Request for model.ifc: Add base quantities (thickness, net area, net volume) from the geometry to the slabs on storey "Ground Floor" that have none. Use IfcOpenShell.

First a look at what the model holds.

```python
import ifcopenshell
import ifcopenshell.util.element
import ifcopenshell.util.unit

model = ifcopenshell.open("model.ifc")
print(model.schema)
for unit_type in ("LENGTHUNIT", "AREAUNIT", "VOLUMEUNIT"):
    print(unit_type, ifcopenshell.util.unit.calculate_unit_scale(model, unit_type))
storey = next(s for s in model.by_type("IfcBuildingStorey") if s.Name == "Ground Floor")
slabs = [e for e in ifcopenshell.util.element.get_decomposition(storey) if e.is_a("IfcSlab")]
for e in sorted(slabs, key=lambda e: e.id()):
    print(e.id(), e.is_a(), e.Name, list(ifcopenshell.util.element.get_psets(e, qtos_only=True)), sep=" | ")
```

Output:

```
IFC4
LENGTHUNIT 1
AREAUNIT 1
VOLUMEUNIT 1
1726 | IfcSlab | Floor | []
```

```python
import ifcopenshell
import ifcopenshell.api.pset
import ifcopenshell.geom
import ifcopenshell.util.element
import ifcopenshell.util.shape
import ifcopenshell.util.unit

model = ifcopenshell.open("model.ifc")
unit_scale = ifcopenshell.util.unit.calculate_unit_scale(model)
area_scale = ifcopenshell.util.unit.calculate_unit_scale(model, "AREAUNIT")
volume_scale = ifcopenshell.util.unit.calculate_unit_scale(model, "VOLUMEUNIT")
settings = ifcopenshell.geom.settings()

storey = next(s for s in model.by_type("IfcBuildingStorey") if s.Name == "Ground Floor")
slabs = [e for e in ifcopenshell.util.element.get_decomposition(storey) if e.is_a("IfcSlab")]

for e in sorted(slabs, key=lambda e: e.id()):
    if ifcopenshell.util.element.get_psets(e, qtos_only=True, should_inherit=False):
        continue
    # Geometry comes back in metres, in the element's own axes.
    shape = ifcopenshell.geom.create_shape(settings, e)
    values = {
        "Width": ifcopenshell.util.shape.get_z(shape.geometry) / unit_scale,
        "NetArea": ifcopenshell.util.shape.get_footprint_area(shape.geometry) / area_scale,
        "NetVolume": ifcopenshell.util.shape.get_volume(shape.geometry) / volume_scale,
    }
    qto = ifcopenshell.api.pset.add_qto(model, product=e, name="Qto_SlabBaseQuantities")
    ifcopenshell.api.pset.edit_qto(model, qto=qto, properties=values)
    print(e.id(), {k: round(v, 3) for k, v in values.items()})

model.write("model_rev.ifc")
```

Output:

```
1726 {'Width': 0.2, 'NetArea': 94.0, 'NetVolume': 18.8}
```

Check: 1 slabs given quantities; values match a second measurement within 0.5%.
